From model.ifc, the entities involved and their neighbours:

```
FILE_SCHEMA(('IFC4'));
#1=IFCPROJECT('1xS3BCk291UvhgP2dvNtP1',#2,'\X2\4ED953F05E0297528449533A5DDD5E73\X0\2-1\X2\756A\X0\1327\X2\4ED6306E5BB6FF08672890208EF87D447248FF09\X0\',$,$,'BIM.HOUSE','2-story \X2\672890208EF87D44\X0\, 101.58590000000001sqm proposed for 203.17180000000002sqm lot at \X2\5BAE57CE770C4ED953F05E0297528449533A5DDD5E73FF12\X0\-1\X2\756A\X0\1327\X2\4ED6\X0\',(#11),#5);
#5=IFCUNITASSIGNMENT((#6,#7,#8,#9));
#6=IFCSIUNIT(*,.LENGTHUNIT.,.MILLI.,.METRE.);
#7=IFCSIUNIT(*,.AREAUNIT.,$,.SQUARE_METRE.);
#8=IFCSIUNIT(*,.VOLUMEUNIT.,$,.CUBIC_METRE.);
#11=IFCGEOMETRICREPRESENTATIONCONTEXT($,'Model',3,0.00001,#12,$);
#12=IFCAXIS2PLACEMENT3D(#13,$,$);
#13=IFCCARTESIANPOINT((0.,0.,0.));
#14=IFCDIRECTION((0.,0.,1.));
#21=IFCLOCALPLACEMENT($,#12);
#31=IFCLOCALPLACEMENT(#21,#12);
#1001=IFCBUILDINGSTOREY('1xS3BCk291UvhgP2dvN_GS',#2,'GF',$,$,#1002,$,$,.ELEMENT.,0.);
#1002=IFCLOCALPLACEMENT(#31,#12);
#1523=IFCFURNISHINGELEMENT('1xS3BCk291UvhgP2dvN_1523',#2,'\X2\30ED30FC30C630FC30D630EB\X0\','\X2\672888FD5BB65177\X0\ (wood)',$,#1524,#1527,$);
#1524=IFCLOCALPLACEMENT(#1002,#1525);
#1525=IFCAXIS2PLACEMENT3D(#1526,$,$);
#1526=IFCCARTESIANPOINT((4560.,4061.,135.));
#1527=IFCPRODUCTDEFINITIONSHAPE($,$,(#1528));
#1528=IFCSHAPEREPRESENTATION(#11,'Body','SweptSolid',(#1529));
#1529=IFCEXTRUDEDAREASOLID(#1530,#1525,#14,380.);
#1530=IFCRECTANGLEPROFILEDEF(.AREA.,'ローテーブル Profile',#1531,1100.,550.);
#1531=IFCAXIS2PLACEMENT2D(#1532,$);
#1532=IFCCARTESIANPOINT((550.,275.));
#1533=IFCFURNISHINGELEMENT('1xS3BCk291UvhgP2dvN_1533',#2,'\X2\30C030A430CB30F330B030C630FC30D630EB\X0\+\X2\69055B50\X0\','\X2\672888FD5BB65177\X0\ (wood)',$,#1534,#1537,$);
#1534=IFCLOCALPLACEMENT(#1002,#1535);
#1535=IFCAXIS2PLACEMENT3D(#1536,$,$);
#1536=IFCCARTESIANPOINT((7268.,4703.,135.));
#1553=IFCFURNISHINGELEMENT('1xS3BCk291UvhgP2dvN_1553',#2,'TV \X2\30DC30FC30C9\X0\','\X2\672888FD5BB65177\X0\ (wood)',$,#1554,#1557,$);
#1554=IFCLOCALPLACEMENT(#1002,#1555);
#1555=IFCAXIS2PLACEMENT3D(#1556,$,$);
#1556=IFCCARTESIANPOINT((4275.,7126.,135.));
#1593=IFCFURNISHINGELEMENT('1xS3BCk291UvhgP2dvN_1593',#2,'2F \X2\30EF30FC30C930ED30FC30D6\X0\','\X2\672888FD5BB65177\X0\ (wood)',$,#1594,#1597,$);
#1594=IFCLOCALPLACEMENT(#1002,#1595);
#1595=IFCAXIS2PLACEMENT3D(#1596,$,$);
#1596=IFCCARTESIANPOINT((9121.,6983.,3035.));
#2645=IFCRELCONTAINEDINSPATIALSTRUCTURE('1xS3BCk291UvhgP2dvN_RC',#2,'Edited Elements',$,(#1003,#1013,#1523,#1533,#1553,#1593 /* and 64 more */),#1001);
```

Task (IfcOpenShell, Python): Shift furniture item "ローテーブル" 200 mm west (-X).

```python
import ifcopenshell
import ifcopenshell.api.geometry
import ifcopenshell.util.placement
import ifcopenshell.util.unit

model = ifcopenshell.open("model.ifc")
unit_scale = ifcopenshell.util.unit.calculate_unit_scale(model)

item = model.by_guid("1xS3BCk291UvhgP2dvN_1523")
matrix = ifcopenshell.util.placement.get_local_placement(item.ObjectPlacement)
matrix[0, 3] -= 0.2 / unit_scale
ifcopenshell.api.geometry.edit_object_placement(model, product=item, matrix=matrix, is_si=False)

print(ifcopenshell.util.placement.get_local_placement(item.ObjectPlacement).round(3) + 0.0)

model.write("model_edited.ifc")
```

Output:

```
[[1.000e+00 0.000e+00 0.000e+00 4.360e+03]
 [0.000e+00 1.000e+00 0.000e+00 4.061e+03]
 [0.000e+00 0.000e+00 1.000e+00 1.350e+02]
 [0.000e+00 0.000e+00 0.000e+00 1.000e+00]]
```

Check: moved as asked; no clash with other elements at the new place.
